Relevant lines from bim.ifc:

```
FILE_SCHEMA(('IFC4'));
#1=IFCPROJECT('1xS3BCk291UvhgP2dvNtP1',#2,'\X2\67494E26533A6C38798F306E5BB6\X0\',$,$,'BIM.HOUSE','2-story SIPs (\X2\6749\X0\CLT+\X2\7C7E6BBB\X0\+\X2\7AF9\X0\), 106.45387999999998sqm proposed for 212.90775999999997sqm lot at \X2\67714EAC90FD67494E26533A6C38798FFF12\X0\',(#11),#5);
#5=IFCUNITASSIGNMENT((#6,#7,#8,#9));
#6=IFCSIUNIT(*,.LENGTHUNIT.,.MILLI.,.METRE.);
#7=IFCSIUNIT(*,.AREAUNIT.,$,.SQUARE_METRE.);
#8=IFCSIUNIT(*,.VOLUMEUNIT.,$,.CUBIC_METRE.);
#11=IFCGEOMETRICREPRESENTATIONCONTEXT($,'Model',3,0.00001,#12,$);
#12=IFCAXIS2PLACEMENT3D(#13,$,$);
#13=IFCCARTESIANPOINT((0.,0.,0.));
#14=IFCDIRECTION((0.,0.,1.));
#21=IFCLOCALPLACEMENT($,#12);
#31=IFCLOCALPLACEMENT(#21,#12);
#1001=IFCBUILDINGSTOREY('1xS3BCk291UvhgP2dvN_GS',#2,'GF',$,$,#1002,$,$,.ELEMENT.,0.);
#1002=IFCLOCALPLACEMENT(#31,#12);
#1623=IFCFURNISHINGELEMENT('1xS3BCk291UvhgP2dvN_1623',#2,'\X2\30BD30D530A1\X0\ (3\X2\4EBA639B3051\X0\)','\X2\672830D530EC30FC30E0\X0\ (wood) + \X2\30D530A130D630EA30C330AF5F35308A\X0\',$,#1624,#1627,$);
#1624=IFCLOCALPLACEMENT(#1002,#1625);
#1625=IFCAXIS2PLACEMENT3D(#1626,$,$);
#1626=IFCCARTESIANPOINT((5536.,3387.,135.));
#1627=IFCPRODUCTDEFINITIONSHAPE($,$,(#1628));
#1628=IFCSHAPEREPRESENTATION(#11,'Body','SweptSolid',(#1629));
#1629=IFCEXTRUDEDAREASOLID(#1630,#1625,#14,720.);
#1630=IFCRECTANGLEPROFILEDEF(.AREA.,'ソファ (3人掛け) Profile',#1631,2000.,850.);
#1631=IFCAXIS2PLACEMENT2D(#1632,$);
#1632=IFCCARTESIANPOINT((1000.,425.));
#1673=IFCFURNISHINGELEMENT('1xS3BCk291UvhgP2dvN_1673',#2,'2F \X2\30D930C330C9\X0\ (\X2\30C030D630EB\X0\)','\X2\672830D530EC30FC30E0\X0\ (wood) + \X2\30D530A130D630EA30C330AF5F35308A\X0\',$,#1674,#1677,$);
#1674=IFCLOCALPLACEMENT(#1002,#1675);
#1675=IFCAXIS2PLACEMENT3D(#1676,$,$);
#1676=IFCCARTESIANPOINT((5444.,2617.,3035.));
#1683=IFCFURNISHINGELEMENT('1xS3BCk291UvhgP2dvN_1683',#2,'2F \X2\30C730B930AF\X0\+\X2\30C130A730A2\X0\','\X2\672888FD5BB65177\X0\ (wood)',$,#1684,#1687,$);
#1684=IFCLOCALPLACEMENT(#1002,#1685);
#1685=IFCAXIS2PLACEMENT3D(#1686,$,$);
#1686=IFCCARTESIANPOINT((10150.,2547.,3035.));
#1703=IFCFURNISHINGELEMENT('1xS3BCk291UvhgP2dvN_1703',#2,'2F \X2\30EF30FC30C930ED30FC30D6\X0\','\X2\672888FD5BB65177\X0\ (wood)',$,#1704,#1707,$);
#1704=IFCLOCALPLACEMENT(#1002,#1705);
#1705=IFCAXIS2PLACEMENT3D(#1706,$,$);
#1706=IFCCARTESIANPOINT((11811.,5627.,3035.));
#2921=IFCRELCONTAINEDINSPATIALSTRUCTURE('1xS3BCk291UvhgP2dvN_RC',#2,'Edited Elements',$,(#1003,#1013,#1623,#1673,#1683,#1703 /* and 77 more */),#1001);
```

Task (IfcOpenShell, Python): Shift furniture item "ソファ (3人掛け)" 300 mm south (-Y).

```python
import ifcopenshell
import ifcopenshell.api.geometry
import ifcopenshell.util.placement
import ifcopenshell.util.unit

model = ifcopenshell.open("bim.ifc")
unit_scale = ifcopenshell.util.unit.calculate_unit_scale(model)

item = model.by_id(1623)
matrix = ifcopenshell.util.placement.get_local_placement(item.ObjectPlacement)
matrix[1, 3] -= 0.3 / unit_scale
ifcopenshell.api.geometry.edit_object_placement(model, product=item, matrix=matrix, is_si=False)

print(ifcopenshell.util.placement.get_local_placement(item.ObjectPlacement).round(3) + 0.0)

model.write("bim-out.ifc")
```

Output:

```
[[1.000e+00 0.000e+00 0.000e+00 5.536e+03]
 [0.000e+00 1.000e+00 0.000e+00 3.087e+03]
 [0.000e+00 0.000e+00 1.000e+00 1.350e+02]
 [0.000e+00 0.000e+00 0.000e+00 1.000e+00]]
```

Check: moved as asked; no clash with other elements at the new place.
